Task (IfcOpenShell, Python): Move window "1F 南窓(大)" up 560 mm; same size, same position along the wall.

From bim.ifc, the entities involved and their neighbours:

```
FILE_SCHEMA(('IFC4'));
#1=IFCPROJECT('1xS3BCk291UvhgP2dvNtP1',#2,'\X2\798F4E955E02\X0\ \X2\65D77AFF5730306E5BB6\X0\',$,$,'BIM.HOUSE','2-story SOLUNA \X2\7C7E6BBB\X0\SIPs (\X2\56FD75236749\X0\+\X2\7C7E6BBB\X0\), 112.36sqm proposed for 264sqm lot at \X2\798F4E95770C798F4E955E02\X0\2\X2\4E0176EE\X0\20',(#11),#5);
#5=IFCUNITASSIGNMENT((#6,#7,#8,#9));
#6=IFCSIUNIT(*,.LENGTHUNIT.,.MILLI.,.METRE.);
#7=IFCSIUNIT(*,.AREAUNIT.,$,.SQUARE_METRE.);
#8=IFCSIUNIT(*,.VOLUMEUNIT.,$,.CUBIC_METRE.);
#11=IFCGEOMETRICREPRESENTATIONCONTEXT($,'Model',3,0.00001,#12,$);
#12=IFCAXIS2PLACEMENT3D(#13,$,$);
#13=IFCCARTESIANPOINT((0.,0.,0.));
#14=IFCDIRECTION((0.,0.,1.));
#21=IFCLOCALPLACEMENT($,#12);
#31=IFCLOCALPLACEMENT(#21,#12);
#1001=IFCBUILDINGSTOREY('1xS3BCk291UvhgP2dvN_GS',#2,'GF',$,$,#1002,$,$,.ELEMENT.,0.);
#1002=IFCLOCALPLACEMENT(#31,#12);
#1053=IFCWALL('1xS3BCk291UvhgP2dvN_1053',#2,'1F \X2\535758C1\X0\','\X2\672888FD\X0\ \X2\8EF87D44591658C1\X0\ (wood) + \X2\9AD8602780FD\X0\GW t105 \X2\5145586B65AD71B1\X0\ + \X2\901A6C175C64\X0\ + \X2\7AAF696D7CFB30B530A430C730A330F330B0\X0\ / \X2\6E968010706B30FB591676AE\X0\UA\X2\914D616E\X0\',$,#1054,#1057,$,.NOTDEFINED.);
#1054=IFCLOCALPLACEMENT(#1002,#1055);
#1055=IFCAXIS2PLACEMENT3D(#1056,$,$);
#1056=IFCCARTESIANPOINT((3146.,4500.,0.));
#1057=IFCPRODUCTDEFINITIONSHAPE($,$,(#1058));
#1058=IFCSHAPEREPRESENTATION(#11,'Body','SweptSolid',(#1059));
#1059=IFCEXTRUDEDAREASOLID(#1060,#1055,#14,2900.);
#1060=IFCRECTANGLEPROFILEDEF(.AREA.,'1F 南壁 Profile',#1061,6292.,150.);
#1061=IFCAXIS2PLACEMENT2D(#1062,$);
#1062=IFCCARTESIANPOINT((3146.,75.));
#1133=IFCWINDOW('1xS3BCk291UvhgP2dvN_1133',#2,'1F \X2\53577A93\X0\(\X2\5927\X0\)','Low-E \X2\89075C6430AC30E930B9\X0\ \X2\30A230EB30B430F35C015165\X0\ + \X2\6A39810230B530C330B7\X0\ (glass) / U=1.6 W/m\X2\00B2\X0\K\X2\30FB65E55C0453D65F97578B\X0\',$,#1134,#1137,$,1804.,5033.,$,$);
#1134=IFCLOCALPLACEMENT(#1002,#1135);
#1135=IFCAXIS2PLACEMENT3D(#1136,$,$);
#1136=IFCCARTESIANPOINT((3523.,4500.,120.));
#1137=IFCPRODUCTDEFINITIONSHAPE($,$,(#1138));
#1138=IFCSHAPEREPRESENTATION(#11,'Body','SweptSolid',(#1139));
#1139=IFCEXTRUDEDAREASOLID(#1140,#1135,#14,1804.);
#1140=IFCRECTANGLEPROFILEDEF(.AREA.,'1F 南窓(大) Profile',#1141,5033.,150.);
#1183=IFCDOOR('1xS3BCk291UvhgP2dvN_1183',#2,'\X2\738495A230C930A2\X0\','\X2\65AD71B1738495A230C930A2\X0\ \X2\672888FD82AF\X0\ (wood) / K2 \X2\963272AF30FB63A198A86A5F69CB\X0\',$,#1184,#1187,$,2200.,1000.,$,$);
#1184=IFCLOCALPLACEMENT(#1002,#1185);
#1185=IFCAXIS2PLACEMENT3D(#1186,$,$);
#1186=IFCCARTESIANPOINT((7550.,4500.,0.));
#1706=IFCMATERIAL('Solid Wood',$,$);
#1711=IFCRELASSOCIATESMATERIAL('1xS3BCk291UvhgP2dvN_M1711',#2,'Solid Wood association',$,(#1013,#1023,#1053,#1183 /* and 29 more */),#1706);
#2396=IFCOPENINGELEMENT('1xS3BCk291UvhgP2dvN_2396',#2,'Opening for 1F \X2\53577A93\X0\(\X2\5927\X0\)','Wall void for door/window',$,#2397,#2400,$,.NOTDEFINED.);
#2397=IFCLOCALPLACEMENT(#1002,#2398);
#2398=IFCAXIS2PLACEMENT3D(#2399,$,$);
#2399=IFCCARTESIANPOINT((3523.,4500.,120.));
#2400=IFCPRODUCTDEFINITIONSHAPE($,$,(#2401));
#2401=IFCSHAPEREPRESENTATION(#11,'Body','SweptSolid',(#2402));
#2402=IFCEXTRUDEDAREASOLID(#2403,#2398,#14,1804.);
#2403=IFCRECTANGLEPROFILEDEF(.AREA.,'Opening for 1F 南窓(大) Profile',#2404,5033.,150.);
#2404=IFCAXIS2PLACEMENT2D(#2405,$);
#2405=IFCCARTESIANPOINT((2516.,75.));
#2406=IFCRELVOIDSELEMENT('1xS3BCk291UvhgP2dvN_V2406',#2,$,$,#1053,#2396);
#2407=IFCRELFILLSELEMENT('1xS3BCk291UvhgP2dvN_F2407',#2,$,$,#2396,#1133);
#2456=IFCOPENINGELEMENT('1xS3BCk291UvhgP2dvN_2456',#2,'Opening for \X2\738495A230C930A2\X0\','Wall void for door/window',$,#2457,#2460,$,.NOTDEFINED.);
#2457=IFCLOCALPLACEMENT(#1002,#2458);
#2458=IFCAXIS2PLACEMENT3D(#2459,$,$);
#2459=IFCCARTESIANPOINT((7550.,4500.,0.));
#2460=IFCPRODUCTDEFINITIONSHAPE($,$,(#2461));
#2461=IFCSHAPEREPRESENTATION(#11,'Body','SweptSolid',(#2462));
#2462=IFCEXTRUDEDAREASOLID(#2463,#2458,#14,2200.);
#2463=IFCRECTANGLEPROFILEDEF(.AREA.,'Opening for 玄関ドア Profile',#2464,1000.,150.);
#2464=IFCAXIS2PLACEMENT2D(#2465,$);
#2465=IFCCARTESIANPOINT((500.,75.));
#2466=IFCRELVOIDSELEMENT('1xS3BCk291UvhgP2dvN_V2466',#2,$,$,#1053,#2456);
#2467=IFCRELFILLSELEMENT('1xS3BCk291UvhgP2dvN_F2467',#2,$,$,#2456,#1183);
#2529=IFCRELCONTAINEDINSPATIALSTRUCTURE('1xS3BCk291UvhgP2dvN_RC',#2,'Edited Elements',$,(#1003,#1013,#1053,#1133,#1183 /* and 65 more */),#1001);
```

```python
import numpy as np
import ifcopenshell
import ifcopenshell.api.geometry
import ifcopenshell.util.placement
import ifcopenshell.util.unit

model = ifcopenshell.open("bim.ifc")
unit_scale = ifcopenshell.util.unit.calculate_unit_scale(model)

window = model.by_guid("1xS3BCk291UvhgP2dvN_1133")
opening = window.FillsVoids[0].RelatingOpeningElement
dz = 560.0

shift = np.array([0.0, 0.0, dz])
# The window is not placed relative to its opening, so move both.
for product in (opening, window):
    matrix = ifcopenshell.util.placement.get_local_placement(product.ObjectPlacement)
    matrix[:3, 3] += shift
    ifcopenshell.api.geometry.edit_object_placement(model, product=product, matrix=matrix, is_si=False)

print(f"moved by {dz * unit_scale:+.3f} m")

model.write("bim_edited.ifc")
```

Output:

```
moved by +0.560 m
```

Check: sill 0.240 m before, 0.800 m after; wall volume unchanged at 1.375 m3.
